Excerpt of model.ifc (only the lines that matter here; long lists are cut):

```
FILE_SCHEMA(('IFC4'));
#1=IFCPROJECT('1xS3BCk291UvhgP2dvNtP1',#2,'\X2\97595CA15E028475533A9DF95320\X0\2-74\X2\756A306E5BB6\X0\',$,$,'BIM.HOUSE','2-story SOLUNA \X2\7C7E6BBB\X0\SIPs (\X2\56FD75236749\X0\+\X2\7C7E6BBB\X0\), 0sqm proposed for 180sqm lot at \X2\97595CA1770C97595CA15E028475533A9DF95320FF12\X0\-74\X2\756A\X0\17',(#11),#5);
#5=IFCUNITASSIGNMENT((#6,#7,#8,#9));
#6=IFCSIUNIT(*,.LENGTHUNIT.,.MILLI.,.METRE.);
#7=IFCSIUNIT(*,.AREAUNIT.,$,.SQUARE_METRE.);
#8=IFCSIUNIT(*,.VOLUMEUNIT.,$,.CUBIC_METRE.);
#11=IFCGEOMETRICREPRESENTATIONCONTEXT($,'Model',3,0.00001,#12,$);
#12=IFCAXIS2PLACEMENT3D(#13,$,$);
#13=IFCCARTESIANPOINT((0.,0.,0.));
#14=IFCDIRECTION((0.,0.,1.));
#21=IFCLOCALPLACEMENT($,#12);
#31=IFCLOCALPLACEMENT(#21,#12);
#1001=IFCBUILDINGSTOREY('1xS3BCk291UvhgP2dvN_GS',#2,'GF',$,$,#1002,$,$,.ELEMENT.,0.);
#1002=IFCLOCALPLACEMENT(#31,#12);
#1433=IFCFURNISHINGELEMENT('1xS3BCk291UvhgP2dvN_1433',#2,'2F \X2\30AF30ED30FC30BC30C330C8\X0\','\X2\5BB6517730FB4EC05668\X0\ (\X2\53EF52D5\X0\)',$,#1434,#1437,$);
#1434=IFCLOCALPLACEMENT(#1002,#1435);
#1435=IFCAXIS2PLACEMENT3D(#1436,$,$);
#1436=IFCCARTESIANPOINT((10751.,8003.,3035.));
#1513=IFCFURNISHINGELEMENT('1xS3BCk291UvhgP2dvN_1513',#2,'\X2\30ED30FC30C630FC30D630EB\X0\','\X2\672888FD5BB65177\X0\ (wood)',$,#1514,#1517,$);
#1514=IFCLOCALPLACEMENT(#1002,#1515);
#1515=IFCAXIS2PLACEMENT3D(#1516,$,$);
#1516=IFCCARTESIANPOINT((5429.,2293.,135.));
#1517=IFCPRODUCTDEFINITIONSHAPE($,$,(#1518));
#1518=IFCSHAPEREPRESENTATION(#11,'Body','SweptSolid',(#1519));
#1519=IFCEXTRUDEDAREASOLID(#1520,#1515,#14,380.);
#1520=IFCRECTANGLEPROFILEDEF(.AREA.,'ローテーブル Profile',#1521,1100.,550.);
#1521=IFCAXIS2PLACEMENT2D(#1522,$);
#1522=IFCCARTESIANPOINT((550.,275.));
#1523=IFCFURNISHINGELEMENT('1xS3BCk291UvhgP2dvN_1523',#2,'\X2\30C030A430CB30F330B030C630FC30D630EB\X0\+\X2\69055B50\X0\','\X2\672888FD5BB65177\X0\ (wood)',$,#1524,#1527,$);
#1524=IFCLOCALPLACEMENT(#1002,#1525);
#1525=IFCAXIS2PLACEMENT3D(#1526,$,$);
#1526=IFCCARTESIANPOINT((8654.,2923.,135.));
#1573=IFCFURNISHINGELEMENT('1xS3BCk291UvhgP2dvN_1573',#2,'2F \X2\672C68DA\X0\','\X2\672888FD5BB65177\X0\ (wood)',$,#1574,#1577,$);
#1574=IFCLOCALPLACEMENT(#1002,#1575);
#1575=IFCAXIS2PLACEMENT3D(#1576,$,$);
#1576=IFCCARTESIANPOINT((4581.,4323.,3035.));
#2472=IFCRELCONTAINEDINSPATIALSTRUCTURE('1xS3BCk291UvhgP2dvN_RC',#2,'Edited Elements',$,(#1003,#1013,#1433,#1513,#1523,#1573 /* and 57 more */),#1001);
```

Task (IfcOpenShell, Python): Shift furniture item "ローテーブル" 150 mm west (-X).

```python
import ifcopenshell
import ifcopenshell.api.geometry
import ifcopenshell.util.placement

model = ifcopenshell.open("model.ifc")

item = model.by_guid("1xS3BCk291UvhgP2dvN_1513")
matrix = ifcopenshell.util.placement.get_local_placement(item.ObjectPlacement)
matrix[0, 3] -= 150.0
ifcopenshell.api.geometry.edit_object_placement(model, product=item, matrix=matrix, is_si=False)

print(ifcopenshell.util.placement.get_local_placement(item.ObjectPlacement).round(3) + 0.0)

model.write("model_updated.ifc")
```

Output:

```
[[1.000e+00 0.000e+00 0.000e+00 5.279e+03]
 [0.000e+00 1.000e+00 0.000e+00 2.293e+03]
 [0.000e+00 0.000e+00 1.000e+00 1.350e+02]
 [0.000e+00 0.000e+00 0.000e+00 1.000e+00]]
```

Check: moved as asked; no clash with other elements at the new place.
